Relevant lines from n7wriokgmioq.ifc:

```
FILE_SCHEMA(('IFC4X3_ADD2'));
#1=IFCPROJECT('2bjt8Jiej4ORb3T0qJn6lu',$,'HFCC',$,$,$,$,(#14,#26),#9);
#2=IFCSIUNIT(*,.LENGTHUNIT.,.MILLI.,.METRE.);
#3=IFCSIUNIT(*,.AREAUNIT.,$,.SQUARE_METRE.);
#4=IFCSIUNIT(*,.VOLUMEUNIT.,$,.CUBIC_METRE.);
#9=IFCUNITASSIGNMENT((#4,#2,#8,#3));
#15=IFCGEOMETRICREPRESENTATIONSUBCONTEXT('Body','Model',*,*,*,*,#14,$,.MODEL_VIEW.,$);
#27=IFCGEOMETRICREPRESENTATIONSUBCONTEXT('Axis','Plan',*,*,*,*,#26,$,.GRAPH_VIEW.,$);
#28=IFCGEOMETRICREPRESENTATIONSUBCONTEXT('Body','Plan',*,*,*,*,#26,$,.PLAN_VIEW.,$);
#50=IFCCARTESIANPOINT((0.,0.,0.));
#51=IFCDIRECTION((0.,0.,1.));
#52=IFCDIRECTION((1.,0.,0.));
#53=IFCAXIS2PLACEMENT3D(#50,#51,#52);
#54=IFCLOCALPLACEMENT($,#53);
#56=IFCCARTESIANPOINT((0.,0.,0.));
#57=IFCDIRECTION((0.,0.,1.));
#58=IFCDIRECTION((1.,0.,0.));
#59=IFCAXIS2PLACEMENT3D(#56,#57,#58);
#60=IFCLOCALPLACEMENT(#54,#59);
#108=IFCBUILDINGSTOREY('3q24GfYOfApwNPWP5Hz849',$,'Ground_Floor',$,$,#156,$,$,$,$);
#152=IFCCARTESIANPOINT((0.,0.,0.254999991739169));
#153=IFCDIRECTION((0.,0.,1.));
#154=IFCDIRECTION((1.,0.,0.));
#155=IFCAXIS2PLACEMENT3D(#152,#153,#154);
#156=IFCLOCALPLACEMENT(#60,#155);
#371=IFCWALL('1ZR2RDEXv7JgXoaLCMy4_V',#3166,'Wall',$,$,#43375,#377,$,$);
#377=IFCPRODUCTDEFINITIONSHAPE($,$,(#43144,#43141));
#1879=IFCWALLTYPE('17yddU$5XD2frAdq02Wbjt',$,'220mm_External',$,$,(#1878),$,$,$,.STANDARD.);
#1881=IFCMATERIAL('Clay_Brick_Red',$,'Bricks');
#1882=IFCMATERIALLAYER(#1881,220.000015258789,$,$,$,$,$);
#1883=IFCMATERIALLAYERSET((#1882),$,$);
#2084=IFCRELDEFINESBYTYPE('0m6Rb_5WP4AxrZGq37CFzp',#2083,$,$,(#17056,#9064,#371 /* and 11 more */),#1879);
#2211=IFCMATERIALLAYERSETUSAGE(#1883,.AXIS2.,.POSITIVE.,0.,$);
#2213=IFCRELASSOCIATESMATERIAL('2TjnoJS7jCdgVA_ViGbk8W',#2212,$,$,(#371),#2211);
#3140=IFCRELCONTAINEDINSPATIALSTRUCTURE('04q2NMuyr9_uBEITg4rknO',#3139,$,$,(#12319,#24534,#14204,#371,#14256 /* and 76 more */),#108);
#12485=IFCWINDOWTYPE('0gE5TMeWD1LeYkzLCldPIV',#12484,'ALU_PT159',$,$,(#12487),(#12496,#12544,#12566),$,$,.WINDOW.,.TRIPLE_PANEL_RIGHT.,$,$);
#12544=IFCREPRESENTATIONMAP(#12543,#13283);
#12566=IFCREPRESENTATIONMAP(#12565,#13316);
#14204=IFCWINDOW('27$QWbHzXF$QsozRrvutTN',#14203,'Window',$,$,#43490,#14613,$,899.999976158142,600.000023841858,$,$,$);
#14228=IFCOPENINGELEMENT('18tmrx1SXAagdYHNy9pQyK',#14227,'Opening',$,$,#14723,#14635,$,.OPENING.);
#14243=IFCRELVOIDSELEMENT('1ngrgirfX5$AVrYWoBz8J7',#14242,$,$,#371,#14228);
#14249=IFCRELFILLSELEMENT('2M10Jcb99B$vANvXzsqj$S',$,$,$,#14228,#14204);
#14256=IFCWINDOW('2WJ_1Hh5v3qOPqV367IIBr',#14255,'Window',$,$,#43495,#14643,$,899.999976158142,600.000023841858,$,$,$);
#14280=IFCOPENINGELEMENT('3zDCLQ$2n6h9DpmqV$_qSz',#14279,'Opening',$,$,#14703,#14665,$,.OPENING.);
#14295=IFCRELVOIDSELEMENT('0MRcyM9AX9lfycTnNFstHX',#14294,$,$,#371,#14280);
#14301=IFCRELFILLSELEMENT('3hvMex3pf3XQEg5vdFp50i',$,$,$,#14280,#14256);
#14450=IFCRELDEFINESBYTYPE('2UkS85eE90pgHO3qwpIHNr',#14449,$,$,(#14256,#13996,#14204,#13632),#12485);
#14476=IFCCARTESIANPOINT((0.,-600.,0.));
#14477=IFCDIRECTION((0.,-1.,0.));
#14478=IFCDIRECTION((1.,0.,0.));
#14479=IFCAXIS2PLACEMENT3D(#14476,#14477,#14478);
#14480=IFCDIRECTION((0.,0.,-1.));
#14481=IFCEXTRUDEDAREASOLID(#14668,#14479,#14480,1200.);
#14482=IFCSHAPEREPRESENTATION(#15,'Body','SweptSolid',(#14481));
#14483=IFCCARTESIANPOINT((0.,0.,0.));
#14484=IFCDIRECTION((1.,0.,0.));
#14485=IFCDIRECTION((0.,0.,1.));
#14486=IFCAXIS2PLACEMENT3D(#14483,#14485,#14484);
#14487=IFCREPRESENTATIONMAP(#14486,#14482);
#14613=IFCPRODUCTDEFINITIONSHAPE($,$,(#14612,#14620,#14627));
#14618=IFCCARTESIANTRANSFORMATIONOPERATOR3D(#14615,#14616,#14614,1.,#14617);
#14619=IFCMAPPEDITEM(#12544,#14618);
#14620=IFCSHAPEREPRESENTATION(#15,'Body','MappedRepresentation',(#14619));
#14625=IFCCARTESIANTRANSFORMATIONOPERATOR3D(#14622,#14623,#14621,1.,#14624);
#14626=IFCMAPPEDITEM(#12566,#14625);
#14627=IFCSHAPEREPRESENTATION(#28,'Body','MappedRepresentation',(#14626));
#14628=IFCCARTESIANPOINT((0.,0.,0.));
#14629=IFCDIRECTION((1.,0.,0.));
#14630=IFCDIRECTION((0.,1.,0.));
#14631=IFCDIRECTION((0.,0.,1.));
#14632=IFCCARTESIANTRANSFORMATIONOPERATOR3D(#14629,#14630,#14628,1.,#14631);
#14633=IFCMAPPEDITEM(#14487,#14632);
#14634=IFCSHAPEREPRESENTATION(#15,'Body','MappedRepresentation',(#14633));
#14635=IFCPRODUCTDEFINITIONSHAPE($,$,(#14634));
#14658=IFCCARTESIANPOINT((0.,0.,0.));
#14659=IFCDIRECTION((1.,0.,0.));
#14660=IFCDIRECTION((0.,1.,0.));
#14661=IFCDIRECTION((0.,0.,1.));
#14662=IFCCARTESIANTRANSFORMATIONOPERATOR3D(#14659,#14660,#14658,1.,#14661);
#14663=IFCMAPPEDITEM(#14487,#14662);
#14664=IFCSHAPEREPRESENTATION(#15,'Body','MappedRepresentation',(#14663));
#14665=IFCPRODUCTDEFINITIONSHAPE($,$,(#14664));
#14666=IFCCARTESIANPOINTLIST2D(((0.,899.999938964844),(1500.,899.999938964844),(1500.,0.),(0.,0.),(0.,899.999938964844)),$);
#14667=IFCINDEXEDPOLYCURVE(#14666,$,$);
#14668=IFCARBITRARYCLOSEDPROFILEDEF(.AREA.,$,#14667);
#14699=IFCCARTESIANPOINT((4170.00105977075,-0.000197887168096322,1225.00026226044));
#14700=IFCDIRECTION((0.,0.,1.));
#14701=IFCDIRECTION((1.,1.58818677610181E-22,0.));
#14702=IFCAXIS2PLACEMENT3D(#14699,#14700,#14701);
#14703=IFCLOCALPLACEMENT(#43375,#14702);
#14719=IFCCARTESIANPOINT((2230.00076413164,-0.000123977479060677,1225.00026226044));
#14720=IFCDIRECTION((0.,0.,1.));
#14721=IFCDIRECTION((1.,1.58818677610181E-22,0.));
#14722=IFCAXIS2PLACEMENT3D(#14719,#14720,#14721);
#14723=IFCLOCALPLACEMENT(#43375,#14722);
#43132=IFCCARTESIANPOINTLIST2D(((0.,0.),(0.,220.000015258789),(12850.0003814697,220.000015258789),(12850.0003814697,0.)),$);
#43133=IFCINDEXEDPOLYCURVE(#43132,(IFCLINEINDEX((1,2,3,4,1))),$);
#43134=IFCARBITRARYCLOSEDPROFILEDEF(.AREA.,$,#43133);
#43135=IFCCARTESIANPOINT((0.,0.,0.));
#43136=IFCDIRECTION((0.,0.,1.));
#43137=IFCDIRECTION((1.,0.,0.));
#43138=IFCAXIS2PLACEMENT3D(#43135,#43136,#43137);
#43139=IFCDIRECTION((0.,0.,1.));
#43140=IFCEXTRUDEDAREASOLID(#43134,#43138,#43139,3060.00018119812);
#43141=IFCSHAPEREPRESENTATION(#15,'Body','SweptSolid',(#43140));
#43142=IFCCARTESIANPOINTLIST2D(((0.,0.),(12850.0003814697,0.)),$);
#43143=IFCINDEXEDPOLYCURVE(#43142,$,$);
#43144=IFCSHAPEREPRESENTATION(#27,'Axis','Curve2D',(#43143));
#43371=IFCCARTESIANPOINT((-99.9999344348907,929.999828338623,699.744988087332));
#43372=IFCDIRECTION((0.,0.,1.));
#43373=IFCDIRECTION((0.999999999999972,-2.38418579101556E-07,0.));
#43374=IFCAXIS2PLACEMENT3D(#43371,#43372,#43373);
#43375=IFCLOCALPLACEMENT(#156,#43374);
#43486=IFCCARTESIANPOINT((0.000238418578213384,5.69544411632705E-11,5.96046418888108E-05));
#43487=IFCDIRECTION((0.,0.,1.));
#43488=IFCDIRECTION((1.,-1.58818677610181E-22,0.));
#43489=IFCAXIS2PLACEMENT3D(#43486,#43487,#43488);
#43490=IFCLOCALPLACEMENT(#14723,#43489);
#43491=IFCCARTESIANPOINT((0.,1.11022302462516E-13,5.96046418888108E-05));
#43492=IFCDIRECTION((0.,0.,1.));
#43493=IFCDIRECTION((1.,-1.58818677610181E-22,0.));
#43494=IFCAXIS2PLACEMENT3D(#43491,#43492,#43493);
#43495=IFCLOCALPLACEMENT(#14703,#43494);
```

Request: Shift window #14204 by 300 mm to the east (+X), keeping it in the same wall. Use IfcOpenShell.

```python
import ifcopenshell
import ifcopenshell.api.geometry
import ifcopenshell.util.placement

model = ifcopenshell.open("n7wriokgmioq.ifc")

window = model.by_id(14204)
opening = window.FillsVoids[0].RelatingOpeningElement
wall = opening.VoidsElements[0].RelatingBuildingElement

wall_matrix = ifcopenshell.util.placement.get_local_placement(wall.ObjectPlacement)
shift = wall_matrix[:3, 0] * 300.0
before = ifcopenshell.util.placement.get_local_placement(window.ObjectPlacement)[:3, 3].copy()

# The window is placed relative to its opening, so it follows when the opening moves.
matrix = ifcopenshell.util.placement.get_local_placement(opening.ObjectPlacement)
matrix[:3, 3] += shift
ifcopenshell.api.geometry.edit_object_placement(
    model, product=opening, matrix=matrix, is_si=False, should_transform_children=True
)

after = ifcopenshell.util.placement.get_local_placement(window.ObjectPlacement)[:3, 3]
print("window moved by", (after - before).round(3) + 0.0)

model.write("n7wriokgmioq_v2.ifc")
```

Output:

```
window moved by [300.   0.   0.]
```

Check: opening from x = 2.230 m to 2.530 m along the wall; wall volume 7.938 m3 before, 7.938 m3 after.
